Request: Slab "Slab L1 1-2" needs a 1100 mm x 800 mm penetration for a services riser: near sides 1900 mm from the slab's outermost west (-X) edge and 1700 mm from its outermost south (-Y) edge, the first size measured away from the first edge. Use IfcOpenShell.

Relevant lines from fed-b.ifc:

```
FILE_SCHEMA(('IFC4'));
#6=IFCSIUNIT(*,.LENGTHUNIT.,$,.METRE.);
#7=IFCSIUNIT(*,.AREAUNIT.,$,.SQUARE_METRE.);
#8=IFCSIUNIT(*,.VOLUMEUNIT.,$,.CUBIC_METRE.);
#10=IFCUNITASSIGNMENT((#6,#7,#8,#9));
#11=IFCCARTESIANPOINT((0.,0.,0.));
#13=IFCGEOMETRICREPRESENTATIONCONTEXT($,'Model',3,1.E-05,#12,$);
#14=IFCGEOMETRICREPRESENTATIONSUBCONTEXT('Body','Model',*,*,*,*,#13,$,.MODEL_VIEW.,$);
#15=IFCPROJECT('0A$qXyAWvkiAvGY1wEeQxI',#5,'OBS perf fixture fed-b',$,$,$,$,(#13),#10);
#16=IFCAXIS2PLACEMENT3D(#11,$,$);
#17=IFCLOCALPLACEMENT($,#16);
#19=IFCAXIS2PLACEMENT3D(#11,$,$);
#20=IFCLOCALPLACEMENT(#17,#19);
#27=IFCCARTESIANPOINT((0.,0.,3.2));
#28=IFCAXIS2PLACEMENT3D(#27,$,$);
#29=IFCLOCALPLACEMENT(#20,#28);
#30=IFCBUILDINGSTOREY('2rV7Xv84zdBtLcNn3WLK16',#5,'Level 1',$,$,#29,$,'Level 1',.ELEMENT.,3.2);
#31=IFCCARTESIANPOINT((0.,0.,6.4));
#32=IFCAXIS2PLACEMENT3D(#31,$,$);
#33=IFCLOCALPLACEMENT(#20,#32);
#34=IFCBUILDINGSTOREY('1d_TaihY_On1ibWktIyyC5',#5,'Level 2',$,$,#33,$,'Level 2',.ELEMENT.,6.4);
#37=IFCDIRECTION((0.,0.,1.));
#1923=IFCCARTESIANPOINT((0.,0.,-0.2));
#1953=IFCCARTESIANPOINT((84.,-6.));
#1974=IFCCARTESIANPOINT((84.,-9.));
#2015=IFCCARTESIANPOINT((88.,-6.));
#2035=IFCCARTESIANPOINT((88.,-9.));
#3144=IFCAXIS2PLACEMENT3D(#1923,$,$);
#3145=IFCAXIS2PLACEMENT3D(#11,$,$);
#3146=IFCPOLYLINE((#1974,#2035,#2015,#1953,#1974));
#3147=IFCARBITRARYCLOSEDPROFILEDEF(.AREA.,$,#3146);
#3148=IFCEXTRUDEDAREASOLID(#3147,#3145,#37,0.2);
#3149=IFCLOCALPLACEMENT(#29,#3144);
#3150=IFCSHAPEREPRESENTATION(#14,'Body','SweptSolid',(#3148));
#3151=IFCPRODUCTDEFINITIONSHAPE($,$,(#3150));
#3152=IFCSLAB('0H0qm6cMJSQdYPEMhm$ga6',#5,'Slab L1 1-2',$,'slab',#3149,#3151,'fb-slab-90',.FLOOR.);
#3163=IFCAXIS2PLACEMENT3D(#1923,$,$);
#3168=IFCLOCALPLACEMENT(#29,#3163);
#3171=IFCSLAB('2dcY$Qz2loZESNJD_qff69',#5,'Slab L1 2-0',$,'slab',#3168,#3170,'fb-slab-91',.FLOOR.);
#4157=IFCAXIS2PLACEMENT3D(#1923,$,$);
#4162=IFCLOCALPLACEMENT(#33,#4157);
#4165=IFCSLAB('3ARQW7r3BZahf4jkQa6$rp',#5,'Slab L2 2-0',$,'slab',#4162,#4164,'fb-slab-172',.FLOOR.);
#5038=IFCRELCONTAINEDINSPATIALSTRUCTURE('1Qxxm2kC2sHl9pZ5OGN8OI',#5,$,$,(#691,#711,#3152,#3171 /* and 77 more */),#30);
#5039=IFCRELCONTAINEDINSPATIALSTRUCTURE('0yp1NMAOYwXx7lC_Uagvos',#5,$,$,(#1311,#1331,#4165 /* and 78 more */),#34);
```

```python
import numpy as np
import ifcopenshell
import ifcopenshell.api.feature
import ifcopenshell.api.geometry
import ifcopenshell.api.root
import ifcopenshell.geom
import ifcopenshell.util.placement
import ifcopenshell.util.representation
import ifcopenshell.util.shape
import ifcopenshell.util.unit

model = ifcopenshell.open("fed-b.ifc")
unit_scale = ifcopenshell.util.unit.calculate_unit_scale(model)
settings = ifcopenshell.geom.settings()


def volume(element):
    """Net volume in cubic metres, openings subtracted."""
    shape = ifcopenshell.geom.create_shape(settings, element)
    return ifcopenshell.util.shape.get_volume(shape.geometry)


slab = model.by_id(3152)
before = volume(slab)

# Extent in the slab's own axes, in metres. The edges named are its -X and -Y sides.
slab_shape = ifcopenshell.geom.create_shape(settings, slab)
vertices = ifcopenshell.util.shape.get_vertices(slab_shape.geometry)
x_min, y_min, bottom = vertices.min(axis=0)
top = vertices[:, 2].max()

opening = ifcopenshell.api.root.create_entity(model, ifc_class="IfcOpeningElement", name="Services riser opening", predefined_type="OPENING")
context = ifcopenshell.util.representation.get_context(model, "Model", "Body", "MODEL_VIEW")
width, depth = 1.1, 0.8
outline = [(0.0, 0.0), (width, 0.0), (width, depth), (0.0, depth), (0.0, 0.0)]
# Overshoot both faces by 50 mm so the cut is clean.
shape = ifcopenshell.api.geometry.add_slab_representation(
    model, context=context, depth=top - bottom + 0.1, polyline=outline
)
ifcopenshell.api.geometry.assign_representation(model, product=opening, representation=shape)

matrix = ifcopenshell.util.placement.get_local_placement(slab.ObjectPlacement)
matrix[:, 3] = matrix @ np.append(np.array([x_min + 1.9, y_min + 1.7, bottom - 0.05]) / unit_scale, 1.0)
ifcopenshell.api.geometry.edit_object_placement(model, product=opening, matrix=matrix, is_si=False)
ifcopenshell.api.feature.add_feature(model, feature=opening, element=slab)

after = volume(slab)

print(f"slab volume {before:.3f} -> {after:.3f} m3")

model.write("fed-b_rev.ifc")
```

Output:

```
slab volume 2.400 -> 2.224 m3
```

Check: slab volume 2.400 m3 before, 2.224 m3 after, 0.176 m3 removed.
